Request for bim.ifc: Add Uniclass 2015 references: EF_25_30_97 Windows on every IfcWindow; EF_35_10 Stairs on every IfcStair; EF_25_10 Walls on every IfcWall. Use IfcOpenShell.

First a look at what the model holds.

```python
import ifcopenshell

model = ifcopenshell.open("bim.ifc")
print(model.schema)
print("classifications:", [c.Name for c in model.by_type("IfcClassification")])
for ifc_class in ("IfcDoor", "IfcRoof", "IfcStair", "IfcWall", "IfcWindow"):
    print(ifc_class, len(model.by_type(ifc_class)))
```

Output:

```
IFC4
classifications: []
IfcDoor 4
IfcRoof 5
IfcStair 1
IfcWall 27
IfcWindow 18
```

```python
import ifcopenshell
import ifcopenshell.api.classification

model = ifcopenshell.open("bim.ifc")

system = ifcopenshell.api.classification.add_classification(model, classification="Uniclass 2015")

codes = {
    "IfcWindow": ("EF_25_30_97", "Windows"),
    "IfcStair": ("EF_35_10", "Stairs"),
    "IfcWall": ("EF_25_10", "Walls"),
}
for ifc_class, (code, name) in codes.items():
    products = model.by_type(ifc_class)
    ifcopenshell.api.classification.add_reference(
        model, products=products, classification=system, identification=code, name=name
    )
    print(code, len(products))

model.write("bim_v2.ifc")
```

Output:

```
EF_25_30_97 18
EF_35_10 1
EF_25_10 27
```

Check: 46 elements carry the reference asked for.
